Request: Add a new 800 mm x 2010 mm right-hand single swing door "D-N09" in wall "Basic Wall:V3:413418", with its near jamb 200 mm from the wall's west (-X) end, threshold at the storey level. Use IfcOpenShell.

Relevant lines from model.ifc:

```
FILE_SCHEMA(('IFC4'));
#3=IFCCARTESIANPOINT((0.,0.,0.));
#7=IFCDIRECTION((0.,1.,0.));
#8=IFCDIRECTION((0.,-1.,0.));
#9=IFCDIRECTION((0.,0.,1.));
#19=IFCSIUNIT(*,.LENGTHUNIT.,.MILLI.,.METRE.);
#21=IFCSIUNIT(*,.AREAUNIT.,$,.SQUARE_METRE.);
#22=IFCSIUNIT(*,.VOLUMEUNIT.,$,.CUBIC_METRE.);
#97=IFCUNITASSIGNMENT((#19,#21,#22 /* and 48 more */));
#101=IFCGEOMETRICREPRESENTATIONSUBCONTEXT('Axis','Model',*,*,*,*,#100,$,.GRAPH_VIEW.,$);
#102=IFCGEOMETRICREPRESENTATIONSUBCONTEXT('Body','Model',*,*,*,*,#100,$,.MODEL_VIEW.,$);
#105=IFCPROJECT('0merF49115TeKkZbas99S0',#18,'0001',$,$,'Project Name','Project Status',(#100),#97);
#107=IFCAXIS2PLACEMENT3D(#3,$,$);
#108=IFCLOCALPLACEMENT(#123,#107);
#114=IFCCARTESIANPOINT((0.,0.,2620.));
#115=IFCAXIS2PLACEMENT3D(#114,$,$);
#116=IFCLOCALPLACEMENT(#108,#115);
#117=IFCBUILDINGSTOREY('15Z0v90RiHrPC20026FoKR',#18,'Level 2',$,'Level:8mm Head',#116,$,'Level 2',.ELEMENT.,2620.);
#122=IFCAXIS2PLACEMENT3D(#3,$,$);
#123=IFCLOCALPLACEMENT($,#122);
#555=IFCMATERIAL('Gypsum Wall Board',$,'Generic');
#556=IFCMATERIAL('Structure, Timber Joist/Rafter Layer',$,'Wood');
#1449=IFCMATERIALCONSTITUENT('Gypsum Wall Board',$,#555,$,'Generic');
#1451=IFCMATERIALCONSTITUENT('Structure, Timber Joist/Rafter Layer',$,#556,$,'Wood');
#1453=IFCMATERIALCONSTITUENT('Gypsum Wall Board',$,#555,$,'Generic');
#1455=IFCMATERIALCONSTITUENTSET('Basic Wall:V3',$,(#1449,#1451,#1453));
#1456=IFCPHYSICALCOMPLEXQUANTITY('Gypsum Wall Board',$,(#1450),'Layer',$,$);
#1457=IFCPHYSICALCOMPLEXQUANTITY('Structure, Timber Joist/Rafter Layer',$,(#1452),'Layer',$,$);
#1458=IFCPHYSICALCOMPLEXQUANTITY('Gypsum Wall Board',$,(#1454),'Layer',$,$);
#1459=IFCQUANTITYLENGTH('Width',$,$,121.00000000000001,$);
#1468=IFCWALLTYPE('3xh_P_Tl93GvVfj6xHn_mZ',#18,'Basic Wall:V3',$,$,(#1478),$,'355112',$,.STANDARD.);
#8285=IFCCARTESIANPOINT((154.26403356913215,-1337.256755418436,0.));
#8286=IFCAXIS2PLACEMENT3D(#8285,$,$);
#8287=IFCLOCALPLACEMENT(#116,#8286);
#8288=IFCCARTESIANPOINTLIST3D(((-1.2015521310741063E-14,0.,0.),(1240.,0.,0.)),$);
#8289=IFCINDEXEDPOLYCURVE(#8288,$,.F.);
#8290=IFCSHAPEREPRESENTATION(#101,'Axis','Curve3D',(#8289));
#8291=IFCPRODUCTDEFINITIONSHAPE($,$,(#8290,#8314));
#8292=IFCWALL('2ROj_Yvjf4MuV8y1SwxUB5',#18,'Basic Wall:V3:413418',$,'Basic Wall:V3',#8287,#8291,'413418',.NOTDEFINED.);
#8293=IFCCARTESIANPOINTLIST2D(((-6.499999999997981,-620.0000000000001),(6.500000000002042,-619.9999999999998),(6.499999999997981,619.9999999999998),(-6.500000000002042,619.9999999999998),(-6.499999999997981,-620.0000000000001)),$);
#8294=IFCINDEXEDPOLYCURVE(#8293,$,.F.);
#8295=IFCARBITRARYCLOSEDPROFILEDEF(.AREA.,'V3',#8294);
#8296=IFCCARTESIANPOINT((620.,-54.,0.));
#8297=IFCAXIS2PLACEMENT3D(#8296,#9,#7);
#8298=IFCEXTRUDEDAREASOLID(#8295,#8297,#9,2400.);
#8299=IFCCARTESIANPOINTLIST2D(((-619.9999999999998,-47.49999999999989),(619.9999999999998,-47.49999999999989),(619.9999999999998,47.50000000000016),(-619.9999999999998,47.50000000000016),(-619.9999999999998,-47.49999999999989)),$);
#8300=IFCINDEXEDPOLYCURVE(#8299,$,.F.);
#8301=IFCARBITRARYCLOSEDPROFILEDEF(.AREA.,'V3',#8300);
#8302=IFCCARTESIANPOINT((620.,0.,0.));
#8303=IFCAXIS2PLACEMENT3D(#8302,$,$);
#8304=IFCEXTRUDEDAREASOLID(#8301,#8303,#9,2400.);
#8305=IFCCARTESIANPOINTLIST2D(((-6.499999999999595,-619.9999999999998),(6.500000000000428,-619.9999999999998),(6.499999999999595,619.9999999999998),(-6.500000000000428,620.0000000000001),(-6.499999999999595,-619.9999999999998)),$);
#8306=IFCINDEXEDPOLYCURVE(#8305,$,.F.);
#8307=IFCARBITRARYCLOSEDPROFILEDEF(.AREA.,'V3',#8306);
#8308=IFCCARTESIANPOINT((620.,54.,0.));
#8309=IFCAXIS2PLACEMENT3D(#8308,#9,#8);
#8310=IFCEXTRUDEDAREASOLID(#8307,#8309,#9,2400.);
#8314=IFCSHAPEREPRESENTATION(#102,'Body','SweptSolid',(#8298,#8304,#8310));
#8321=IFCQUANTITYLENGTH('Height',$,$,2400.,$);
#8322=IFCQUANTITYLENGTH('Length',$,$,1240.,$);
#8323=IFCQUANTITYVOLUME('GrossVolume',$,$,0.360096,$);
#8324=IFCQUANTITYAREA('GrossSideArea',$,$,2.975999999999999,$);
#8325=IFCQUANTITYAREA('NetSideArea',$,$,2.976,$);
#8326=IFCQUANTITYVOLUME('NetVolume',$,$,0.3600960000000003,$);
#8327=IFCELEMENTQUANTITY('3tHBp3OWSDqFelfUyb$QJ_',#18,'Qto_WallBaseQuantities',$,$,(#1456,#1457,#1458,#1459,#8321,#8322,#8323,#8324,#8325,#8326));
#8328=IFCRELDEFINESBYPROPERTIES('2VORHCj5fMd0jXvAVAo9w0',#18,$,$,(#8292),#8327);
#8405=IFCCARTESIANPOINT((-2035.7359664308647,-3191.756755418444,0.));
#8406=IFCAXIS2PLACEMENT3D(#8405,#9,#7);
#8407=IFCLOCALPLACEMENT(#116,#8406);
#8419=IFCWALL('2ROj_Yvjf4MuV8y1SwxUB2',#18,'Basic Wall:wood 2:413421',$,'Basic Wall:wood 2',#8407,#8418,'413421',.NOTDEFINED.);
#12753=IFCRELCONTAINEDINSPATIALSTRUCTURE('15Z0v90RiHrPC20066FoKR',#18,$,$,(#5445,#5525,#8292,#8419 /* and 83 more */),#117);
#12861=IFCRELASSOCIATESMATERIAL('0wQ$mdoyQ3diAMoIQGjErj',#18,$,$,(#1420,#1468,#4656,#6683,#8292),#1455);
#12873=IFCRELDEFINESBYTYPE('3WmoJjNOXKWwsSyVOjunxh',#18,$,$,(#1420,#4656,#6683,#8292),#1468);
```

```python
import numpy as np
import ifcopenshell
import ifcopenshell.api.feature
import ifcopenshell.api.geometry
import ifcopenshell.api.pset
import ifcopenshell.api.root
import ifcopenshell.api.spatial
import ifcopenshell.geom
import ifcopenshell.util.element
import ifcopenshell.util.placement
import ifcopenshell.util.representation
import ifcopenshell.util.shape
import ifcopenshell.util.unit

model = ifcopenshell.open("model.ifc")
unit_scale = ifcopenshell.util.unit.calculate_unit_scale(model)
area_scale = ifcopenshell.util.unit.calculate_unit_scale(model, "AREAUNIT")
volume_scale = ifcopenshell.util.unit.calculate_unit_scale(model, "VOLUMEUNIT")
settings = ifcopenshell.geom.settings()


def volume(element):
    """Net volume in cubic metres, openings subtracted."""
    shape = ifcopenshell.geom.create_shape(settings, element)
    return ifcopenshell.util.shape.get_volume(shape.geometry)


wall = model.by_guid("2ROj_Yvjf4MuV8y1SwxUB5")
storey = ifcopenshell.util.element.get_container(wall, ifc_class="IfcBuildingStorey")
context = ifcopenshell.util.representation.get_context(model, "Model", "Body", "MODEL_VIEW")
before = volume(wall)

width, height, from_end, sill = 0.8, 2.01, 0.2, 0.0  # metres

# The wall runs along its own X axis, and the end named is its -X end.
wall_shape = ifcopenshell.geom.create_shape(settings, wall)
x, y, z = ifcopenshell.util.shape.get_vertices(wall_shape.geometry).T
start = x.min() + from_end
face, thickness = float(y.min()), float(y.max() - y.min())
wall_matrix = ifcopenshell.util.placement.get_local_placement(wall.ObjectPlacement)
level = ifcopenshell.util.placement.get_local_placement(storey.ObjectPlacement)[2, 3]


def in_wall(x, y):
    """Placement at x, y metres in the wall's axes, at sill height."""
    matrix = wall_matrix.copy()
    matrix[:, 3] = wall_matrix @ np.array([x / unit_scale, y / unit_scale, 0.0, 1.0])
    matrix[2, 3] = level + sill / unit_scale
    return matrix


# Opening: a box that overshoots both wall faces by 50 mm.
opening = ifcopenshell.api.root.create_entity(model, ifc_class="IfcOpeningElement", predefined_type="OPENING")
box = ifcopenshell.api.geometry.add_wall_representation(
    model, context=context, length=width, height=height, thickness=thickness + 0.1
)
ifcopenshell.api.geometry.assign_representation(model, product=opening, representation=box)
ifcopenshell.api.geometry.edit_object_placement(model, product=opening, matrix=in_wall(start, face - 0.05), is_si=False)
ifcopenshell.api.feature.add_feature(model, feature=opening, element=wall)

door = ifcopenshell.api.root.create_entity(model, ifc_class="IfcDoor", name="D-N09", predefined_type="DOOR")
door.OverallWidth, door.OverallHeight = width / unit_scale, height / unit_scale
door.OperationType = "SINGLE_SWING_RIGHT"
body = ifcopenshell.api.geometry.add_door_representation(
    model,
    context=context,
    overall_width=door.OverallWidth,
    overall_height=door.OverallHeight,
    operation_type="SINGLE_SWING_RIGHT",
    lining_properties={"LiningDepth": thickness / unit_scale, "ThresholdDepth": thickness / unit_scale},
)
ifcopenshell.api.geometry.assign_representation(model, product=door, representation=body)
ifcopenshell.api.spatial.assign_container(model, products=[door], relating_structure=storey)
ifcopenshell.api.feature.add_filling(model, opening=opening, element=door)

# The lining spans the wall, so the door starts at the wall face.
ifcopenshell.api.geometry.edit_object_placement(model, product=door, matrix=in_wall(start, face), is_si=False)

after = volume(wall)

# Update the wall's stored quantities.
qto = model.by_id(ifcopenshell.util.element.get_pset(wall, "Qto_WallBaseQuantities", should_inherit=False)["id"])
ifcopenshell.api.pset.edit_qto(model, qto=qto, properties={
    "NetSideArea": after / thickness / area_scale,
    "NetVolume": after / volume_scale,
})

print(f"wall volume {before:.3f} -> {after:.3f} m3")

model.write("model_edited.ifc")
```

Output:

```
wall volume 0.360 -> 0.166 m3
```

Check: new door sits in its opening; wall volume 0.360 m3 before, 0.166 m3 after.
